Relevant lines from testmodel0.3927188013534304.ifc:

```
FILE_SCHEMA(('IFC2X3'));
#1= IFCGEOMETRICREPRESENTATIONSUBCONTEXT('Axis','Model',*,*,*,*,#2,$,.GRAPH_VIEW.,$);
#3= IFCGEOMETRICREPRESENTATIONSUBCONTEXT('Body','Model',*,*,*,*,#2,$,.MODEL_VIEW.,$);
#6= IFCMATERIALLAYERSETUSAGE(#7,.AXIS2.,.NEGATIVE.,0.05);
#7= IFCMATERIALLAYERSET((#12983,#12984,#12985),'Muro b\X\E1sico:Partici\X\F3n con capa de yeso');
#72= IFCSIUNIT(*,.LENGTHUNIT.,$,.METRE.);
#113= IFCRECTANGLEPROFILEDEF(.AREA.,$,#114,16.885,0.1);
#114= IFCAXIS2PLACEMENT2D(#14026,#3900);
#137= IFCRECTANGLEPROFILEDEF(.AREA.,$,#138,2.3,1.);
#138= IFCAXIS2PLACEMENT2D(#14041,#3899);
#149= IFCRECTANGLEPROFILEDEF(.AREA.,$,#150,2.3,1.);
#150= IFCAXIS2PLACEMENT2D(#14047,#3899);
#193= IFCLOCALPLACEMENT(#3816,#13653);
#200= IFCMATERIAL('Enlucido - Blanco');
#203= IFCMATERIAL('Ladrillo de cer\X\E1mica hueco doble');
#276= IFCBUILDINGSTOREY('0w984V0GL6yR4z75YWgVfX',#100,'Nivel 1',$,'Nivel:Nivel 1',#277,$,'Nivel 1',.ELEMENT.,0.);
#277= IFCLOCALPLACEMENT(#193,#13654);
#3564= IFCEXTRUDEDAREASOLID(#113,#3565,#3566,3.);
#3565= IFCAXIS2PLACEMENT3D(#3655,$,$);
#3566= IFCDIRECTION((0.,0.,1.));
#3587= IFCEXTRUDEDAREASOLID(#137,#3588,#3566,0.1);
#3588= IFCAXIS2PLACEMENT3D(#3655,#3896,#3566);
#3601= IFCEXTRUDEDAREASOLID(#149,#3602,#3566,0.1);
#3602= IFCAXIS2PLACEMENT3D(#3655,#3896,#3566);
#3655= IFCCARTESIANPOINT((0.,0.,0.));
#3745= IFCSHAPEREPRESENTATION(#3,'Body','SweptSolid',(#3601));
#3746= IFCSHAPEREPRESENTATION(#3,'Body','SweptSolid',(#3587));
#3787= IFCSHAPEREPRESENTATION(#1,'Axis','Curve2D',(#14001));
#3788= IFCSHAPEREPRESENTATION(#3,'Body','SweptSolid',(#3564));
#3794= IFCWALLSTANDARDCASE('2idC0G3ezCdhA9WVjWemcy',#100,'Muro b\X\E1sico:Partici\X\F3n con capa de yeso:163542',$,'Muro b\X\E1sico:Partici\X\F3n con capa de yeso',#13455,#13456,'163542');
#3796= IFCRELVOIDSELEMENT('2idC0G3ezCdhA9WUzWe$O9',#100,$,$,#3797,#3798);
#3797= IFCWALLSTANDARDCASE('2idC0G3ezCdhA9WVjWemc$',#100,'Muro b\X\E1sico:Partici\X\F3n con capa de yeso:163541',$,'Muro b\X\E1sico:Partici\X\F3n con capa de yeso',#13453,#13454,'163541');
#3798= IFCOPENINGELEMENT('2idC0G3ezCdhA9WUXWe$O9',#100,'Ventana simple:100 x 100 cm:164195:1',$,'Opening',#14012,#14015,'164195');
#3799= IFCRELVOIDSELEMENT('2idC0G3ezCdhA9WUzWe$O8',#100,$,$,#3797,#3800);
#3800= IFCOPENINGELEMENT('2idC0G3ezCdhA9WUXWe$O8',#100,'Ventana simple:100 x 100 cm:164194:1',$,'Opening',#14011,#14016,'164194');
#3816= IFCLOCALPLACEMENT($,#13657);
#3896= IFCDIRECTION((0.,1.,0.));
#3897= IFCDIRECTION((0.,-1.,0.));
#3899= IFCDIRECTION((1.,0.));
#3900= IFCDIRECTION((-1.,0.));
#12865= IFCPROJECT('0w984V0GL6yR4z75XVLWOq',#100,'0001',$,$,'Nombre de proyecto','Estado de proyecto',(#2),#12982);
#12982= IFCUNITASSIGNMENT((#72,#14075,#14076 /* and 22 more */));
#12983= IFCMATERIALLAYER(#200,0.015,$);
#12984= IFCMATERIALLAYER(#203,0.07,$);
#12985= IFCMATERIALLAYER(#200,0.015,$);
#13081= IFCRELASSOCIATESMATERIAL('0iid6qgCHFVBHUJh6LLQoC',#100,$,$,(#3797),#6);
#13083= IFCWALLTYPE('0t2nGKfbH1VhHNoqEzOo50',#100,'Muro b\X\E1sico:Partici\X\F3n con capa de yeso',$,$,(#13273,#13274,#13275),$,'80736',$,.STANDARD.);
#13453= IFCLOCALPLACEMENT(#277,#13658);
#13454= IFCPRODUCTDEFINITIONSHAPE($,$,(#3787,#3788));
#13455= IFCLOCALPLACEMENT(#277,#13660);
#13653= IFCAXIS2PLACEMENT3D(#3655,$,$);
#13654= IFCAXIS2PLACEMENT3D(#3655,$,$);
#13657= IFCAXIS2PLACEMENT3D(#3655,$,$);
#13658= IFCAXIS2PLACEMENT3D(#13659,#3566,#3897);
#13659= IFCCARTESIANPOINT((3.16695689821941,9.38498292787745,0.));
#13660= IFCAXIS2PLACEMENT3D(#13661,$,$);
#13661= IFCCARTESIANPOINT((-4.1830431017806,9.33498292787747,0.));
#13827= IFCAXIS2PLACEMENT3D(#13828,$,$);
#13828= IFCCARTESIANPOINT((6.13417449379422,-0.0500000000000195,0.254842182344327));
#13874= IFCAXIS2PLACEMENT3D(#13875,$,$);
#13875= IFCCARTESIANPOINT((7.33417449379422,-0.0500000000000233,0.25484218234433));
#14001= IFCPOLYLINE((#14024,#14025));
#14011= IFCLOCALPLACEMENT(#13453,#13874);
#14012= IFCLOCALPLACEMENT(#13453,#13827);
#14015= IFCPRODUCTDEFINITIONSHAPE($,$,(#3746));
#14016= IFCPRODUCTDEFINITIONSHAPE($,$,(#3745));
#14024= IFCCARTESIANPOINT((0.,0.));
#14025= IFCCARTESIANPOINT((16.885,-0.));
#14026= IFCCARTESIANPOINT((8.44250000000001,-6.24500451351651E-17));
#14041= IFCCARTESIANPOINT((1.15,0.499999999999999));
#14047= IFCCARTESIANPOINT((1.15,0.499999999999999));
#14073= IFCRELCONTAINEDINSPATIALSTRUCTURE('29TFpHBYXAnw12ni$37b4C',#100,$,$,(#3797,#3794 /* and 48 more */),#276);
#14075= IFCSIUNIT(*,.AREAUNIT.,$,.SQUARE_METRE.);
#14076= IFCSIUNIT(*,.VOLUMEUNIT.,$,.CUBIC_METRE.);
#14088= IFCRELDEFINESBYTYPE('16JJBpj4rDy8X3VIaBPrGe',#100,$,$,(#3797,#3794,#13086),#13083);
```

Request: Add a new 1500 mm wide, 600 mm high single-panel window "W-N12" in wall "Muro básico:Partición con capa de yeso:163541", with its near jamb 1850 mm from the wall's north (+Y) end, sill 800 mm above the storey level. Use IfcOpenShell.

```python
import numpy as np
import ifcopenshell
import ifcopenshell.api.feature
import ifcopenshell.api.geometry
import ifcopenshell.api.root
import ifcopenshell.api.spatial
import ifcopenshell.api.type
import ifcopenshell.geom
import ifcopenshell.util.element
import ifcopenshell.util.placement
import ifcopenshell.util.representation
import ifcopenshell.util.shape
import ifcopenshell.util.unit

model = ifcopenshell.open("testmodel0.3927188013534304.ifc")
unit_scale = ifcopenshell.util.unit.calculate_unit_scale(model)
settings = ifcopenshell.geom.settings()


def volume(element):
    """Net volume in cubic metres, openings subtracted."""
    shape = ifcopenshell.geom.create_shape(settings, element)
    return ifcopenshell.util.shape.get_volume(shape.geometry)


wall = model.by_guid("2idC0G3ezCdhA9WVjWemc$")
storey = ifcopenshell.util.element.get_container(wall, ifc_class="IfcBuildingStorey")
context = ifcopenshell.util.representation.get_context(model, "Model", "Body", "MODEL_VIEW")
before = volume(wall)

width, height, from_end, sill = 1.5, 0.6, 1.85, 0.8  # metres

# The wall runs along its own X axis, and the end named is its -X end.
wall_shape = ifcopenshell.geom.create_shape(settings, wall)
x, y, z = ifcopenshell.util.shape.get_vertices(wall_shape.geometry).T
start = x.min() + from_end
face, thickness = float(y.min()), float(y.max() - y.min())
wall_matrix = ifcopenshell.util.placement.get_local_placement(wall.ObjectPlacement)
level = ifcopenshell.util.placement.get_local_placement(storey.ObjectPlacement)[2, 3]


def in_wall(x, y):
    """Placement at x, y metres in the wall's axes, at sill height."""
    matrix = wall_matrix.copy()
    matrix[:, 3] = wall_matrix @ np.array([x / unit_scale, y / unit_scale, 0.0, 1.0])
    matrix[2, 3] = level + sill / unit_scale
    return matrix


# Opening: a box that overshoots both wall faces by 50 mm.
opening = ifcopenshell.api.root.create_entity(model, ifc_class="IfcOpeningElement")
box = ifcopenshell.api.geometry.add_wall_representation(
    model, context=context, length=width, height=height, thickness=thickness + 0.1
)
ifcopenshell.api.geometry.assign_representation(model, product=opening, representation=box)
ifcopenshell.api.geometry.edit_object_placement(model, product=opening, matrix=in_wall(start, face - 0.05), is_si=False)
ifcopenshell.api.feature.add_feature(model, feature=opening, element=wall)

window = ifcopenshell.api.root.create_entity(model, ifc_class="IfcWindow", name="W-N12")
window.OverallWidth, window.OverallHeight = width / unit_scale, height / unit_scale
body = ifcopenshell.api.geometry.add_window_representation(
    model,
    context=context,
    overall_width=window.OverallWidth,
    overall_height=window.OverallHeight,
    partition_type="SINGLE_PANEL",
)
ifcopenshell.api.geometry.assign_representation(model, product=window, representation=body)
ifcopenshell.api.spatial.assign_container(model, products=[window], relating_structure=storey)
fills = ifcopenshell.api.feature.add_filling(model, opening=opening, element=window)
fills.OwnerHistory = window.OwnerHistory  # required in IFC2X3

# IFC2X3 keeps the operation on the window style.
style = ifcopenshell.api.root.create_entity(model, ifc_class="IfcWindowStyle", name="W-N12")
style.OperationType, style.ConstructionType = "SINGLE_PANEL", "NOTDEFINED"
style.ParameterTakesPrecedence = style.Sizeable = False
ifcopenshell.api.type.assign_type(model, related_objects=[window], relating_type=style)

# Centre the window in the wall's thickness.
ifcopenshell.api.geometry.edit_object_placement(model, product=window, matrix=in_wall(start, face), is_si=False)
window_shape = ifcopenshell.geom.create_shape(settings, window)
depth = ifcopenshell.util.shape.get_vertices(window_shape.geometry)[:, 1]
offset = face + thickness / 2 - (depth.min() + depth.max()) / 2
ifcopenshell.api.geometry.edit_object_placement(model, product=window, matrix=in_wall(start, offset), is_si=False)

after = volume(wall)

print(f"wall volume {before:.3f} -> {after:.3f} m3")

model.write("testmodel0.3927188013534304_rev.ifc")
```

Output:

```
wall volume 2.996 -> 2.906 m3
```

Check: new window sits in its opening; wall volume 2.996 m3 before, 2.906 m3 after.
